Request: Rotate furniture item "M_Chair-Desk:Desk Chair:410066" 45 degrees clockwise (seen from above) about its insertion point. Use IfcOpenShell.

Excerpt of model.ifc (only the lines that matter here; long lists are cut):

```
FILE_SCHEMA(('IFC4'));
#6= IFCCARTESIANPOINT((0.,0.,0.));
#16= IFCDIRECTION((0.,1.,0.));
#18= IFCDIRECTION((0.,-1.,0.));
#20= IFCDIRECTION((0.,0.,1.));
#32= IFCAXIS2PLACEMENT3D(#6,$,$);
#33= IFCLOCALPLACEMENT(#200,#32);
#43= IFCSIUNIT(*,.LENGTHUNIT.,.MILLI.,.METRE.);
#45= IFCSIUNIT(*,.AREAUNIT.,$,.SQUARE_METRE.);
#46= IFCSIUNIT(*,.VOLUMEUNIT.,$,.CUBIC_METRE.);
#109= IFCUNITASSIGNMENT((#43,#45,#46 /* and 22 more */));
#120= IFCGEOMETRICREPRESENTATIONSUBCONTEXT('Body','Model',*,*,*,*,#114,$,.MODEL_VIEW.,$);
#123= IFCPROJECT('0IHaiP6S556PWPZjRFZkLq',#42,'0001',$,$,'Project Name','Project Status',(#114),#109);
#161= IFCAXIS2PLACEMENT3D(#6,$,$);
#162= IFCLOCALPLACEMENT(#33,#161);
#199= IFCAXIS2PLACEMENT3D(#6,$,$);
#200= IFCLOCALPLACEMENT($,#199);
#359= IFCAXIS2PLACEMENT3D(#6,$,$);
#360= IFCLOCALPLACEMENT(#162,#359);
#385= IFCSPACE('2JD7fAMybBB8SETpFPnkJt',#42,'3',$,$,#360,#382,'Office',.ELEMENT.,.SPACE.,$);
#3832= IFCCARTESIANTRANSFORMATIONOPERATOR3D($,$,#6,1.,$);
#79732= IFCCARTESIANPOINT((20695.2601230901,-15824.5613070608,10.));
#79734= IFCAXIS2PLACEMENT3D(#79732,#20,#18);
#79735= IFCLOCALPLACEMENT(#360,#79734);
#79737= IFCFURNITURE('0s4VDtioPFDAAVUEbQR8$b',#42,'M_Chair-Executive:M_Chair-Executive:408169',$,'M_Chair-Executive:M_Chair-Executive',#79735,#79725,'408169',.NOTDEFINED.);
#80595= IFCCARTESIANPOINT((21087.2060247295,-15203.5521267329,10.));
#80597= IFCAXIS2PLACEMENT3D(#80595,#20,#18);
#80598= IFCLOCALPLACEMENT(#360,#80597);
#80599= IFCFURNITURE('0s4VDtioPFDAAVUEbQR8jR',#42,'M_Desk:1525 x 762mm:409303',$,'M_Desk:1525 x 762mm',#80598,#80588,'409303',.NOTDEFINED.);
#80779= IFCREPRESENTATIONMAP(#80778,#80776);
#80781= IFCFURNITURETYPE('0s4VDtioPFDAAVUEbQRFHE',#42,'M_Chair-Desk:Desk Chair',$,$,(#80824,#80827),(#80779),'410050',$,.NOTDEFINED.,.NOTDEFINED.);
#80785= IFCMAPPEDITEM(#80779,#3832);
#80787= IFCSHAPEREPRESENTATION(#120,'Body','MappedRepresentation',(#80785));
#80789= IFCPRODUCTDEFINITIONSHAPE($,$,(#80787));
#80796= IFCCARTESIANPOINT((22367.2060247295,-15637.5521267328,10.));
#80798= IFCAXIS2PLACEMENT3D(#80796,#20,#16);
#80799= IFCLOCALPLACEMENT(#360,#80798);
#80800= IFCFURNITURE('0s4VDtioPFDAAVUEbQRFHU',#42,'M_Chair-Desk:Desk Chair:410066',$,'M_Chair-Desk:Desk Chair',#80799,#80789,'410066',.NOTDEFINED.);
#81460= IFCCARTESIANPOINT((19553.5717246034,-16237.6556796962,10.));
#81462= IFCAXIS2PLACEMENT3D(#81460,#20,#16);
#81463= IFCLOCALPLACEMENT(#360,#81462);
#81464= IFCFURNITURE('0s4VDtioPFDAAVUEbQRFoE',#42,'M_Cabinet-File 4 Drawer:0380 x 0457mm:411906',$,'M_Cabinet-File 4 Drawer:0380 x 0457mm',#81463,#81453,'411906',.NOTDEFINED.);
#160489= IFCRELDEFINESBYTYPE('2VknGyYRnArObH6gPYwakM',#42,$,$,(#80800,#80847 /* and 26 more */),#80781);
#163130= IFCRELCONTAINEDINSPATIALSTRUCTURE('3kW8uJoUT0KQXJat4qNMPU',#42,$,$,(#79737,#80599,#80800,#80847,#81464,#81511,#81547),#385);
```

```python
import ifcopenshell
import ifcopenshell.api.geometry
import ifcopenshell.util.placement

model = ifcopenshell.open("model.ifc")

item = model.by_id(80800)
matrix = ifcopenshell.util.placement.get_local_placement(item.ObjectPlacement)
matrix = matrix @ ifcopenshell.util.placement.rotation(-45, "Z")
ifcopenshell.api.geometry.edit_object_placement(model, product=item, matrix=matrix, is_si=False)

print(ifcopenshell.util.placement.get_local_placement(item.ObjectPlacement).round(3) + 0.0)

model.write("model_rev.ifc")
```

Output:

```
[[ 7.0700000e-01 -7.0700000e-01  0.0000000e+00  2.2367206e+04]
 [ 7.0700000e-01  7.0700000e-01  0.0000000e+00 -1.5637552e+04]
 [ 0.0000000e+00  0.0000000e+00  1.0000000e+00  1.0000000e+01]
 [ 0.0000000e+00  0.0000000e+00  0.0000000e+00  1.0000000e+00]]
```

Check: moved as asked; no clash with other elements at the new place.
